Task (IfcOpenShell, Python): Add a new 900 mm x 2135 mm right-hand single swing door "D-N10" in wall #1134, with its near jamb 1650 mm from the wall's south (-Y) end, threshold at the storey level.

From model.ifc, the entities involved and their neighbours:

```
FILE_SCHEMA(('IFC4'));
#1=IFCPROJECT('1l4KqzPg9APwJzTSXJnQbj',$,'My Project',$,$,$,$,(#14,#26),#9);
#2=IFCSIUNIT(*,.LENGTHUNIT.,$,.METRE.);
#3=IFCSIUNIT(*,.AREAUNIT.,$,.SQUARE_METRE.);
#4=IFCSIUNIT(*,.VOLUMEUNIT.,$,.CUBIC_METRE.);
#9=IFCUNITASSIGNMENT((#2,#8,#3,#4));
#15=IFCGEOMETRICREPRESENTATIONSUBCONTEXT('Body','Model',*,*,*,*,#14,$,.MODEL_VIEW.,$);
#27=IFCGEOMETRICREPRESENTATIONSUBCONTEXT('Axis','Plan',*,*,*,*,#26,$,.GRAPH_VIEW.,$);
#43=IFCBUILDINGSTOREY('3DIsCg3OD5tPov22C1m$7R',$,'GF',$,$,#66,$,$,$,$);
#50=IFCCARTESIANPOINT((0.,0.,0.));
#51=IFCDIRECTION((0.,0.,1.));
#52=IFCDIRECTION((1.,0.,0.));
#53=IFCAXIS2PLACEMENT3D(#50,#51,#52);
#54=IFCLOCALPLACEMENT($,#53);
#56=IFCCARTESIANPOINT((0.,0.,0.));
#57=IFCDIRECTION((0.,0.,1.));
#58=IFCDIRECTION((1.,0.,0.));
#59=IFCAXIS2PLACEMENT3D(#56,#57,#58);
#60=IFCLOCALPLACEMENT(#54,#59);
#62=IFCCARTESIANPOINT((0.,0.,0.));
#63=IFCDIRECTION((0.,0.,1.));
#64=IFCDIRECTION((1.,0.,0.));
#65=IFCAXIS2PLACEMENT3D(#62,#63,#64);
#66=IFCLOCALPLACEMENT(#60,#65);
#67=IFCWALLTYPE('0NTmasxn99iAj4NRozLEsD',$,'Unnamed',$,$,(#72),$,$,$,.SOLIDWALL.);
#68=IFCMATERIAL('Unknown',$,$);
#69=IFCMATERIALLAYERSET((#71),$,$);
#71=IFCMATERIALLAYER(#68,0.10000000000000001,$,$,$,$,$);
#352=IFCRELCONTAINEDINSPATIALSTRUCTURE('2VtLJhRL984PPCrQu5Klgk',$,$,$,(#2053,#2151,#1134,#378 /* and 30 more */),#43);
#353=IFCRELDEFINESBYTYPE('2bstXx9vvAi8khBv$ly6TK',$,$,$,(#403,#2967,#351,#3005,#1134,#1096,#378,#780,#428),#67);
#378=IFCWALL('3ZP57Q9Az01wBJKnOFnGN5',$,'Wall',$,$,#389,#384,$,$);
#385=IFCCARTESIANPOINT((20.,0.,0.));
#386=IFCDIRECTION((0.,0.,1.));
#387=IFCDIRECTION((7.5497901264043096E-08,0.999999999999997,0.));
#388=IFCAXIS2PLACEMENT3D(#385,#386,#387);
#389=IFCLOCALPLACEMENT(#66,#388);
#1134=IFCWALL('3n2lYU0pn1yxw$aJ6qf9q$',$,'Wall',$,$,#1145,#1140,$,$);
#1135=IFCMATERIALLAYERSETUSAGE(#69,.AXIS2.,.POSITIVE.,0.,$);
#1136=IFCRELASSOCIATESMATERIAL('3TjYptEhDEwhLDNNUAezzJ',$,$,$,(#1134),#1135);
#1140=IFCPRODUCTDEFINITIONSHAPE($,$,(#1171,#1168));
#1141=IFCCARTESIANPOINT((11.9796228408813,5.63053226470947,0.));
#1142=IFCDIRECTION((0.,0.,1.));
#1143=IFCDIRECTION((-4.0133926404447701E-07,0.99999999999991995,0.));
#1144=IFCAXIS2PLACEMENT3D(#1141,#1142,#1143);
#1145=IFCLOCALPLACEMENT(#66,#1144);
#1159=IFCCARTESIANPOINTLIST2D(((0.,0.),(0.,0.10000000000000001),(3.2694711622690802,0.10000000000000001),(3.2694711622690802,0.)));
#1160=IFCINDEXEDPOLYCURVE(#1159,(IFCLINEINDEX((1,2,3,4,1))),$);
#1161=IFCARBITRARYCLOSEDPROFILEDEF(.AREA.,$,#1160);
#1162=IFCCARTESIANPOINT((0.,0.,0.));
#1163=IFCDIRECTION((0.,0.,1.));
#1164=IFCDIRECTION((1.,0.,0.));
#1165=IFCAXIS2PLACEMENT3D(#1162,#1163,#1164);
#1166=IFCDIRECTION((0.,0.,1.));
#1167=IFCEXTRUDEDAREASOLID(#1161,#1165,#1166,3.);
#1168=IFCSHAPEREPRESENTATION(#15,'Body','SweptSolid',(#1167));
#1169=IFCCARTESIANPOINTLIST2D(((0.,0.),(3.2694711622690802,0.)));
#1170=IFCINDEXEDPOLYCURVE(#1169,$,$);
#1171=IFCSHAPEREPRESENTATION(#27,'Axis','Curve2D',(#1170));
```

```python
import numpy as np
import ifcopenshell
import ifcopenshell.api.feature
import ifcopenshell.api.geometry
import ifcopenshell.api.root
import ifcopenshell.api.spatial
import ifcopenshell.geom
import ifcopenshell.util.element
import ifcopenshell.util.placement
import ifcopenshell.util.representation
import ifcopenshell.util.shape
import ifcopenshell.util.unit

model = ifcopenshell.open("model.ifc")
unit_scale = ifcopenshell.util.unit.calculate_unit_scale(model)
settings = ifcopenshell.geom.settings()


def volume(element):
    """Net volume in cubic metres, openings subtracted."""
    shape = ifcopenshell.geom.create_shape(settings, element)
    return ifcopenshell.util.shape.get_volume(shape.geometry)


wall = model.by_id(1134)
storey = ifcopenshell.util.element.get_container(wall, ifc_class="IfcBuildingStorey")
context = ifcopenshell.util.representation.get_context(model, "Model", "Body", "MODEL_VIEW")
before = volume(wall)

width, height, from_end, sill = 0.9, 2.135, 1.65, 0.0  # metres

# The wall runs along its own X axis, and the end named is its -X end.
wall_shape = ifcopenshell.geom.create_shape(settings, wall)
x, y, z = ifcopenshell.util.shape.get_vertices(wall_shape.geometry).T
start = x.min() + from_end
face, thickness = float(y.min()), float(y.max() - y.min())
wall_matrix = ifcopenshell.util.placement.get_local_placement(wall.ObjectPlacement)
level = ifcopenshell.util.placement.get_local_placement(storey.ObjectPlacement)[2, 3]


def in_wall(x, y):
    """Placement at x, y metres in the wall's axes, at sill height."""
    matrix = wall_matrix.copy()
    matrix[:, 3] = wall_matrix @ np.array([x / unit_scale, y / unit_scale, 0.0, 1.0])
    matrix[2, 3] = level + sill / unit_scale
    return matrix


# Opening: a box that overshoots both wall faces by 50 mm.
opening = ifcopenshell.api.root.create_entity(model, ifc_class="IfcOpeningElement", predefined_type="OPENING")
box = ifcopenshell.api.geometry.add_wall_representation(
    model, context=context, length=width, height=height, thickness=thickness + 0.1
)
ifcopenshell.api.geometry.assign_representation(model, product=opening, representation=box)
ifcopenshell.api.geometry.edit_object_placement(model, product=opening, matrix=in_wall(start, face - 0.05), is_si=False)
ifcopenshell.api.feature.add_feature(model, feature=opening, element=wall)

door = ifcopenshell.api.root.create_entity(model, ifc_class="IfcDoor", name="D-N10", predefined_type="DOOR")
door.OverallWidth, door.OverallHeight = width / unit_scale, height / unit_scale
door.OperationType = "SINGLE_SWING_RIGHT"
body = ifcopenshell.api.geometry.add_door_representation(
    model,
    context=context,
    overall_width=door.OverallWidth,
    overall_height=door.OverallHeight,
    operation_type="SINGLE_SWING_RIGHT",
    lining_properties={"LiningDepth": thickness / unit_scale, "ThresholdDepth": thickness / unit_scale},
)
ifcopenshell.api.geometry.assign_representation(model, product=door, representation=body)
ifcopenshell.api.spatial.assign_container(model, products=[door], relating_structure=storey)
ifcopenshell.api.feature.add_filling(model, opening=opening, element=door)

# The lining spans the wall, so the door starts at the wall face.
ifcopenshell.api.geometry.edit_object_placement(model, product=door, matrix=in_wall(start, face), is_si=False)

after = volume(wall)

print(f"wall volume {before:.3f} -> {after:.3f} m3")

model.write("model-out.ifc")
```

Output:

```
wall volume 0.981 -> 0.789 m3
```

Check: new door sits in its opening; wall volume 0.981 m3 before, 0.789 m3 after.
